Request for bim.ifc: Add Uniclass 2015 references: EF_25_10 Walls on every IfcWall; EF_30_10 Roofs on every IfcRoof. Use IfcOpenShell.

First a look at what the model holds.

```python
import ifcopenshell

model = ifcopenshell.open("bim.ifc")
print(model.schema)
print("classifications:", [c.Name for c in model.by_type("IfcClassification")])
for ifc_class in ("IfcDoor", "IfcRoof", "IfcStair", "IfcWall", "IfcWindow"):
    print(ifc_class, len(model.by_type(ifc_class)))
```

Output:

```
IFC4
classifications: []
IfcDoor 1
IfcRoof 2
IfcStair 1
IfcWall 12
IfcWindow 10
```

```python
import ifcopenshell
import ifcopenshell.api.classification

model = ifcopenshell.open("bim.ifc")

system = ifcopenshell.api.classification.add_classification(model, classification="Uniclass 2015")

codes = {
    "IfcWall": ("EF_25_10", "Walls"),
    "IfcRoof": ("EF_30_10", "Roofs"),
}
for ifc_class, (code, name) in codes.items():
    products = model.by_type(ifc_class)
    ifcopenshell.api.classification.add_reference(
        model, products=products, classification=system, identification=code, name=name
    )
    print(code, len(products))

model.write("bim_edited.ifc")
```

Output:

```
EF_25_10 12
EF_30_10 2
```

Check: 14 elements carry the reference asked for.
